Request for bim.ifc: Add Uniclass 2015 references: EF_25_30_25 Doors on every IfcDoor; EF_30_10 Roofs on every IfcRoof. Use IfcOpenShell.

First a look at what the model holds.

```python
import ifcopenshell

model = ifcopenshell.open("bim.ifc")
print(model.schema)
print("classifications:", [c.Name for c in model.by_type("IfcClassification")])
for ifc_class in ("IfcDoor", "IfcRoof", "IfcStair", "IfcWall", "IfcWindow"):
    print(ifc_class, len(model.by_type(ifc_class)))
```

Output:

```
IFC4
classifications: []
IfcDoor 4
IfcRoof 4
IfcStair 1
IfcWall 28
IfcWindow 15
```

```python
import ifcopenshell
import ifcopenshell.api.classification

model = ifcopenshell.open("bim.ifc")

system = ifcopenshell.api.classification.add_classification(model, classification="Uniclass 2015")

codes = {
    "IfcDoor": ("EF_25_30_25", "Doors"),
    "IfcRoof": ("EF_30_10", "Roofs"),
}
for ifc_class, (code, name) in codes.items():
    products = model.by_type(ifc_class)
    ifcopenshell.api.classification.add_reference(
        model, products=products, classification=system, identification=code, name=name
    )
    print(code, len(products))

model.write("bim-out.ifc")
```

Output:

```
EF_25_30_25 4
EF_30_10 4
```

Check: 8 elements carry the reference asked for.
